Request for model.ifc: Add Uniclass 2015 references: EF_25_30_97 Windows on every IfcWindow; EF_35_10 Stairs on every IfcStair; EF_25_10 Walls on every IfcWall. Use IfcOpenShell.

First a look at what the model holds.

```python
import ifcopenshell

model = ifcopenshell.open("model.ifc")
print(model.schema)
print("classifications:", [c.Name for c in model.by_type("IfcClassification")])
for ifc_class in ("IfcDoor", "IfcRoof", "IfcStair", "IfcWall", "IfcWindow"):
    print(ifc_class, len(model.by_type(ifc_class)))
```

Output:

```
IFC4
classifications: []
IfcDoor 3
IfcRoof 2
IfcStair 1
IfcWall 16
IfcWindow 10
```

```python
import ifcopenshell
import ifcopenshell.api.classification

model = ifcopenshell.open("model.ifc")

system = ifcopenshell.api.classification.add_classification(model, classification="Uniclass 2015")

codes = {
    "IfcWindow": ("EF_25_30_97", "Windows"),
    "IfcStair": ("EF_35_10", "Stairs"),
    "IfcWall": ("EF_25_10", "Walls"),
}
for ifc_class, (code, name) in codes.items():
    products = model.by_type(ifc_class)
    ifcopenshell.api.classification.add_reference(
        model, products=products, classification=system, identification=code, name=name
    )
    print(code, len(products))

model.write("model_edited.ifc")
```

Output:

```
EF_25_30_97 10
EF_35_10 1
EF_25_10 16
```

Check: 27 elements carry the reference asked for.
